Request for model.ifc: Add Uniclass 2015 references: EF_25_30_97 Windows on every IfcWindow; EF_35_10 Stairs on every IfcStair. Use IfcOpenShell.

First a look at what the model holds.

```python
import ifcopenshell

model = ifcopenshell.open("model.ifc")
print(model.schema)
print("classifications:", [c.Name for c in model.by_type("IfcClassification")])
for ifc_class in ("IfcDoor", "IfcRoof", "IfcStair", "IfcWall", "IfcWindow"):
    print(ifc_class, len(model.by_type(ifc_class)))
```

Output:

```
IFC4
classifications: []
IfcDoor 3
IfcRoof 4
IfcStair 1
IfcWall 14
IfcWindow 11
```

```python
import ifcopenshell
import ifcopenshell.api.classification

model = ifcopenshell.open("model.ifc")

system = ifcopenshell.api.classification.add_classification(model, classification="Uniclass 2015")

codes = {
    "IfcWindow": ("EF_25_30_97", "Windows"),
    "IfcStair": ("EF_35_10", "Stairs"),
}
for ifc_class, (code, name) in codes.items():
    products = model.by_type(ifc_class)
    ifcopenshell.api.classification.add_reference(
        model, products=products, classification=system, identification=code, name=name
    )
    print(code, len(products))

model.write("model-out.ifc")
```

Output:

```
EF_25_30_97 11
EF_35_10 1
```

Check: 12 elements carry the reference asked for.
